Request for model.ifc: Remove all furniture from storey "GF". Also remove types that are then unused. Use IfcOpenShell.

First a look at what the model holds.

```python
import ifcopenshell
import ifcopenshell.util.element

model = ifcopenshell.open("model.ifc")
print(model.schema)
storey = next(s for s in model.by_type("IfcBuildingStorey") if s.Name == "GF")
furniture = [e for e in ifcopenshell.util.element.get_decomposition(storey) if e.is_a("IfcFurnishingElement")]
seen = {}
for e in furniture:
    element_type = ifcopenshell.util.element.get_type(e)
    name = element_type.Name if element_type not in (None, e) else None
    seen[name] = seen.get(name, 0) + 1
for name, count in sorted(seen.items(), key=str):
    print(count, "x", name)
```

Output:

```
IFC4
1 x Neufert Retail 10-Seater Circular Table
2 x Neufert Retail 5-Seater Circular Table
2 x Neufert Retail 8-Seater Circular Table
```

```python
import ifcopenshell
import ifcopenshell.api.root
import ifcopenshell.util.element

model = ifcopenshell.open("model.ifc")

storey = next(s for s in model.by_type("IfcBuildingStorey") if s.Name == "GF")
furniture = [e for e in ifcopenshell.util.element.get_decomposition(storey) if e.is_a("IfcFurnishingElement")]
types = {ifcopenshell.util.element.get_type(e) for e in furniture} - {None, *furniture}

for e in furniture:
    ifcopenshell.api.root.remove_product(model, product=e)
print(len(furniture), "removed")

unused = [t for t in types if not ifcopenshell.util.element.get_types(t)]
for t in unused:
    ifcopenshell.api.root.remove_product(model, product=t)
print(len(unused), "unused types removed")

model.write("model_updated.ifc")
```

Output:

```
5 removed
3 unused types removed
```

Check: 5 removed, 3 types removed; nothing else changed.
